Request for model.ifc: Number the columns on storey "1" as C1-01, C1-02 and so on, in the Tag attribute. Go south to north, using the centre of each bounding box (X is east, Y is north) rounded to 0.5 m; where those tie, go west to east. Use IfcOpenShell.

First a look at what the model holds.

```python
import ifcopenshell
import ifcopenshell.util.element
import ifcopenshell.util.placement

model = ifcopenshell.open("model.ifc")
print(model.schema)
storey = next(s for s in model.by_type("IfcBuildingStorey") if s.Name == "1")
columns = [e for e in ifcopenshell.util.element.get_decomposition(storey) if e.is_a("IfcColumn")]
for e in sorted(columns, key=lambda e: e.id()):
    origin = ifcopenshell.util.placement.get_local_placement(e.ObjectPlacement)[:3, 3]
    print(e.id(), e.Tag, e.Name, origin.round(2) + 0.0, sep=" | ")
```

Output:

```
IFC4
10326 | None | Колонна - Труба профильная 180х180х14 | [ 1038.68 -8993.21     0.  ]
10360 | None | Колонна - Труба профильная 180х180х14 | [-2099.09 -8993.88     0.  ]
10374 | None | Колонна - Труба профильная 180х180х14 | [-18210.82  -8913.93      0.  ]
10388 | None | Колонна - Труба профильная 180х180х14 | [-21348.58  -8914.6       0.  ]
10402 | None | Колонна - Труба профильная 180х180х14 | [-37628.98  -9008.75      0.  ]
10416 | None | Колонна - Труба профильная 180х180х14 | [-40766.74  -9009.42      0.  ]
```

```python
import ifcopenshell
import ifcopenshell.geom
import ifcopenshell.util.element
import ifcopenshell.util.shape

model = ifcopenshell.open("model.ifc")
settings = ifcopenshell.geom.settings()
settings.set("use-world-coords", True)


def centre(element):
    shape = ifcopenshell.geom.create_shape(settings, element)
    return ifcopenshell.util.shape.get_bbox_centroid(shape.geometry)


storey = next(s for s in model.by_type("IfcBuildingStorey") if s.Name == "1")
columns = [e for e in ifcopenshell.util.element.get_decomposition(storey) if e.is_a("IfcColumn")]

# Insertion points can sit at a corner or the storey origin, so sort by the geometry (in metres).
centres = {e: centre(e) for e in columns}
columns.sort(key=lambda e: (round(centres[e][1] / 0.5), centres[e][0]))

for i, e in enumerate(columns, start=1):
    number = f"C1-{i:02d}"
    e.Tag = number
    print(e.id(), number)

model.write("model_v2.ifc")
```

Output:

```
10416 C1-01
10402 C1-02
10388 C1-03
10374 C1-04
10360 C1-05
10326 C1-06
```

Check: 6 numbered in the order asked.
